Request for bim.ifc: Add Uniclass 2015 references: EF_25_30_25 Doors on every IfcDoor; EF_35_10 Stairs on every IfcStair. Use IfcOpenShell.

First a look at what the model holds.

```python
import ifcopenshell

model = ifcopenshell.open("bim.ifc")
print(model.schema)
print("classifications:", [c.Name for c in model.by_type("IfcClassification")])
for ifc_class in ("IfcDoor", "IfcRoof", "IfcStair", "IfcWall", "IfcWindow"):
    print(ifc_class, len(model.by_type(ifc_class)))
```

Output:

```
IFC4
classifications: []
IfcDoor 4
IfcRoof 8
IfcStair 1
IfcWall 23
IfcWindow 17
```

```python
import ifcopenshell
import ifcopenshell.api.classification

model = ifcopenshell.open("bim.ifc")

system = ifcopenshell.api.classification.add_classification(model, classification="Uniclass 2015")

codes = {
    "IfcDoor": ("EF_25_30_25", "Doors"),
    "IfcStair": ("EF_35_10", "Stairs"),
}
for ifc_class, (code, name) in codes.items():
    products = model.by_type(ifc_class)
    ifcopenshell.api.classification.add_reference(
        model, products=products, classification=system, identification=code, name=name
    )
    print(code, len(products))

model.write("bim-out.ifc")
```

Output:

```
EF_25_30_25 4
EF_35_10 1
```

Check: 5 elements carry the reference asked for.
